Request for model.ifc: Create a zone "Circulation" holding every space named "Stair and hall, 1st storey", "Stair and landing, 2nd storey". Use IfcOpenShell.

First a look at what the model holds.

```python
import ifcopenshell

model = ifcopenshell.open("model.ifc")
print(model.schema)
seen = {}
for space in model.by_type("IfcSpace"):
    seen[space.LongName] = seen.get(space.LongName, 0) + 1
for name, count in sorted(seen.items(), key=str):
    print(count, "x", name)
print("zones:", [z.Name for z in model.by_type("IfcZone")][:20])
```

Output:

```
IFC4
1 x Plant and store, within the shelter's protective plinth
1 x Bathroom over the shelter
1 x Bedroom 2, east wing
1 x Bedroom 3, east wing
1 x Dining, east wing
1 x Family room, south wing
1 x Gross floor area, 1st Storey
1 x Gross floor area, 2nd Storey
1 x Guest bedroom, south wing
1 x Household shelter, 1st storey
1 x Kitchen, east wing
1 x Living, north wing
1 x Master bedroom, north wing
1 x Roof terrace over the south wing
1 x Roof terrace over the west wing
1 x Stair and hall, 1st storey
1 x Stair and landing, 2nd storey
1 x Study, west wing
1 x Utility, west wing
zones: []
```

```python
import ifcopenshell
import ifcopenshell.api.group
import ifcopenshell.api.root

model = ifcopenshell.open("model.ifc")

names = {"Stair and hall, 1st storey", "Stair and landing, 2nd storey"}
spaces = [s for s in model.by_type("IfcSpace") if s.LongName in names]

zone = ifcopenshell.api.root.create_entity(model, ifc_class="IfcZone", name="Circulation")
ifcopenshell.api.group.assign_group(model, products=spaces, group=zone)
print(len(spaces), "spaces in", zone.Name)

model.write("model-out.ifc")
```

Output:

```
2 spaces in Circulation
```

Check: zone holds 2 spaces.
